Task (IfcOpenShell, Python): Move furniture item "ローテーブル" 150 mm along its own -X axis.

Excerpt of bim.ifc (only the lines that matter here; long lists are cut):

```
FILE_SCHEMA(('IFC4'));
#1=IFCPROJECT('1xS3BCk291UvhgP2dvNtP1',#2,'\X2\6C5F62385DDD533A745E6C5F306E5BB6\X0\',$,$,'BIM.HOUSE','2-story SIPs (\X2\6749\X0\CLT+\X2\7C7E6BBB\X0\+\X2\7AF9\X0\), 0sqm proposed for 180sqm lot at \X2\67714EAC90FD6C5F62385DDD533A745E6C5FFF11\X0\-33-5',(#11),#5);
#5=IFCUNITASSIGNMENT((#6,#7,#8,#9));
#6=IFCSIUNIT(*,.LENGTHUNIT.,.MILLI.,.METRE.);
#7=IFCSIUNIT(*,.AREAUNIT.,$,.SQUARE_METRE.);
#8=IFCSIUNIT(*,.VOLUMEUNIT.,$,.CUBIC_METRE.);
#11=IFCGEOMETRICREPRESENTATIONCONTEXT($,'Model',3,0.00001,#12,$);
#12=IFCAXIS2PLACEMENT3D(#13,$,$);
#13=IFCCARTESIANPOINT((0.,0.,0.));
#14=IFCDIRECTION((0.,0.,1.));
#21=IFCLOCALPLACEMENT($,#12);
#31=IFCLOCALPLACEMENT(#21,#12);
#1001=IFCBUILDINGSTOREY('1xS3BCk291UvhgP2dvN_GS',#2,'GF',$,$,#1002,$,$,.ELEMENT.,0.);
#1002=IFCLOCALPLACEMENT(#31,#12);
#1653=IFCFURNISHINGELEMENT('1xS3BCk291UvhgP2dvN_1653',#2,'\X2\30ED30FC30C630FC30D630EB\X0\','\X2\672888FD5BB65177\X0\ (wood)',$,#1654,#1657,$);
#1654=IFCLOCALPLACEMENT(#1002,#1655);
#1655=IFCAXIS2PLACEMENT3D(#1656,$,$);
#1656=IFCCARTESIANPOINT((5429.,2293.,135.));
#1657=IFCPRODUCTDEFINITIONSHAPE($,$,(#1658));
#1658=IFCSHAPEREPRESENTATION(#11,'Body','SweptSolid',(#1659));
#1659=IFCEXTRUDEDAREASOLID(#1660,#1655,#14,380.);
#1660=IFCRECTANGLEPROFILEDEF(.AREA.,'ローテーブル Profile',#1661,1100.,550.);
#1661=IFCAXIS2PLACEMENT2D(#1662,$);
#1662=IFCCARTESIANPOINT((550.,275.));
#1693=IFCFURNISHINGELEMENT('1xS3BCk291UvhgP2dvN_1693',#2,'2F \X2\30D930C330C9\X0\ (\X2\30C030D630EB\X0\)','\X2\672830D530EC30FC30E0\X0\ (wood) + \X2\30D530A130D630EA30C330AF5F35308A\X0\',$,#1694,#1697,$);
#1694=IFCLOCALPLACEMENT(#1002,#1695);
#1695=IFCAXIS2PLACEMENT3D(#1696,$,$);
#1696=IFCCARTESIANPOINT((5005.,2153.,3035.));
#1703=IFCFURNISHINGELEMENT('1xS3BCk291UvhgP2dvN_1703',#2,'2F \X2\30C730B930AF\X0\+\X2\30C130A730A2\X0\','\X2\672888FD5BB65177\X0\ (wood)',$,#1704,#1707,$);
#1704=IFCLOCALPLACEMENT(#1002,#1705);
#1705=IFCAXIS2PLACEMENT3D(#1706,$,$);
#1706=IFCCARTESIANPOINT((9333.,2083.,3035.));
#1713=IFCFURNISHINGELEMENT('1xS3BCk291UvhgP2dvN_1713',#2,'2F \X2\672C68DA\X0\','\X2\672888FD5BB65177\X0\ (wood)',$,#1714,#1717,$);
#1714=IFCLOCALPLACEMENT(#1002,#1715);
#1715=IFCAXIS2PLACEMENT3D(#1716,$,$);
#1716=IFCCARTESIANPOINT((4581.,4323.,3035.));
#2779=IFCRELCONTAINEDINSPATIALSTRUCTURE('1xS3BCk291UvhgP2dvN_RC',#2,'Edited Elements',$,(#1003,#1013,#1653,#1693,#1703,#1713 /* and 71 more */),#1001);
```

```python
import ifcopenshell
import ifcopenshell.api.geometry
import ifcopenshell.util.placement
import ifcopenshell.util.unit

model = ifcopenshell.open("bim.ifc")
unit_scale = ifcopenshell.util.unit.calculate_unit_scale(model)

item = model.by_guid("1xS3BCk291UvhgP2dvN_1653")
matrix = ifcopenshell.util.placement.get_local_placement(item.ObjectPlacement)
matrix[:3, 3] -= matrix[:3, 0] * 0.15 / unit_scale
ifcopenshell.api.geometry.edit_object_placement(model, product=item, matrix=matrix, is_si=False)

print(ifcopenshell.util.placement.get_local_placement(item.ObjectPlacement).round(3) + 0.0)

model.write("bim-out.ifc")
```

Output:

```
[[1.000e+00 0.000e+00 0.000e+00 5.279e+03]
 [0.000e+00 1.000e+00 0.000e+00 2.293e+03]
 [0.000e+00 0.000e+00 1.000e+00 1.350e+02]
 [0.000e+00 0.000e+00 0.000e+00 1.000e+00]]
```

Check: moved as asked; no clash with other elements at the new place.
